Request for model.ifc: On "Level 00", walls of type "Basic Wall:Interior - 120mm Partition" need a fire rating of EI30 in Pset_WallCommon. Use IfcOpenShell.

First a look at what the model holds.

```python
import ifcopenshell
import ifcopenshell.util.element

model = ifcopenshell.open("model.ifc")
print(model.schema)
storey = next(s for s in model.by_type("IfcBuildingStorey") if s.Name == "Level 00")
walls = [e for e in ifcopenshell.util.element.get_decomposition(storey) if e.is_a("IfcWall")]
seen = {}
for e in walls:
    element_type = ifcopenshell.util.element.get_type(e)
    key = (element_type.Name if element_type != e and element_type else None, ifcopenshell.util.element.get_pset(e, "Pset_WallCommon", "FireRating"))
    seen[key] = seen.get(key, 0) + 1
for (name, value), count in sorted(seen.items(), key=str):
    print(count, "x", name, "|", value)
```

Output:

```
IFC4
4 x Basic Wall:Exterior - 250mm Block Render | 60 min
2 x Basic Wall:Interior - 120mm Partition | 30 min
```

```python
import ifcopenshell
import ifcopenshell.api.pset
import ifcopenshell.util.element

model = ifcopenshell.open("model.ifc")

storey = next(s for s in model.by_type("IfcBuildingStorey") if s.Name == "Level 00")
walls = [e for e in ifcopenshell.util.element.get_decomposition(storey) if e.is_a("IfcWall")]

count = 0
for e in walls:
    element_type = ifcopenshell.util.element.get_type(e)
    if element_type in (None, e) or element_type.Name != "Basic Wall:Interior - 120mm Partition":
        continue
    # add_pset returns the element's existing set when there is one.
    pset = ifcopenshell.api.pset.add_pset(model, product=e, name="Pset_WallCommon")
    ifcopenshell.api.pset.edit_pset(model, pset=pset, properties={"FireRating": "EI30"})
    count += 1

print(count, "walls updated")

model.write("model_rev.ifc")
```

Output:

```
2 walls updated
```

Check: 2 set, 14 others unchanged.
